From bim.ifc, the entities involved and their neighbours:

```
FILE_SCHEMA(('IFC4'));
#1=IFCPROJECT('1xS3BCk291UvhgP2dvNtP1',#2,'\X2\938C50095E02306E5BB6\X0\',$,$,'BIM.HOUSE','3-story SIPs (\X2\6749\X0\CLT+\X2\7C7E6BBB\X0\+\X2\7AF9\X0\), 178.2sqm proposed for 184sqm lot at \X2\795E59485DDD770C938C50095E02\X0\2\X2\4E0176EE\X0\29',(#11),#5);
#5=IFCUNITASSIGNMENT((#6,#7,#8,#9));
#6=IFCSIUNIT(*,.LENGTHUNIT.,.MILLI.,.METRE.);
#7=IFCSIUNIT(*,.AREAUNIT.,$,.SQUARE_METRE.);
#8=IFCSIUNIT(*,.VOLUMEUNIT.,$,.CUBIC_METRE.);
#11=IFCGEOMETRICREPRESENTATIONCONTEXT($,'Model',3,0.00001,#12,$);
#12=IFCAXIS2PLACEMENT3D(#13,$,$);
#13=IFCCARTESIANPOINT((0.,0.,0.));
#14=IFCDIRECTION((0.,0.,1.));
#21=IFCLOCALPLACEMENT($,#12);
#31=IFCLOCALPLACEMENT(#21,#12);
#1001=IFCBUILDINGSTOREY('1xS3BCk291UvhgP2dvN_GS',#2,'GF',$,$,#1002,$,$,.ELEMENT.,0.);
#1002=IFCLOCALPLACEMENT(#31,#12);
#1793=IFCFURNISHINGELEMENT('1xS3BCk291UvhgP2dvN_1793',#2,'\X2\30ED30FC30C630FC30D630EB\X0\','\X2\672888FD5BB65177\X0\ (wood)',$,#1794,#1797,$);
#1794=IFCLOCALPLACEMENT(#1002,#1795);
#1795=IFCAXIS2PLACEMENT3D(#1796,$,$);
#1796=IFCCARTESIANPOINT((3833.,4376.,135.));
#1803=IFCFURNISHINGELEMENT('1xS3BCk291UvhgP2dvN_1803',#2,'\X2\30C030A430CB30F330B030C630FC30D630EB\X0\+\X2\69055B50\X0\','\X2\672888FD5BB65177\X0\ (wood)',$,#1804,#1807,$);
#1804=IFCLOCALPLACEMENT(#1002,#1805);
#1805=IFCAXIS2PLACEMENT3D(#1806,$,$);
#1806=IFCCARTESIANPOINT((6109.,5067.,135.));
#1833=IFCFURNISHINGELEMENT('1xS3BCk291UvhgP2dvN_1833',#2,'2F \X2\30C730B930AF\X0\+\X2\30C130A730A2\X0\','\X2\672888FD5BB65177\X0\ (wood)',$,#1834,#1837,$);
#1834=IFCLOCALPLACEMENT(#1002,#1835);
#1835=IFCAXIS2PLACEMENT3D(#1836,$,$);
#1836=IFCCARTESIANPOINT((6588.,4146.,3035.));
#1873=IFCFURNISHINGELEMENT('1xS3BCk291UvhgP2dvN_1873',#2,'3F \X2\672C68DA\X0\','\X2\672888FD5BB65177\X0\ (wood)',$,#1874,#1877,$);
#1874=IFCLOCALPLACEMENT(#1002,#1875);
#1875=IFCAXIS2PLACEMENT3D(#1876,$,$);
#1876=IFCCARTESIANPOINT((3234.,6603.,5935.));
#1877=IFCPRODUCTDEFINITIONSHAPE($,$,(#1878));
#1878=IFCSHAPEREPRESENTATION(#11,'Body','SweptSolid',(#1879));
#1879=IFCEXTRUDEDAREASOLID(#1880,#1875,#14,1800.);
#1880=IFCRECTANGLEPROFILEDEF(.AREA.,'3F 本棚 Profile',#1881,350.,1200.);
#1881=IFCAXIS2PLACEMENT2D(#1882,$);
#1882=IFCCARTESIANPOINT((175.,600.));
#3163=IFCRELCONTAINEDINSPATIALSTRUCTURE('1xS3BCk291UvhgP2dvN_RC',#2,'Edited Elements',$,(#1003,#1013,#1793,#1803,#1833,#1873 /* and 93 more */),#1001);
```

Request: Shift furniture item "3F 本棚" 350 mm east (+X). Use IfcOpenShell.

```python
import ifcopenshell
import ifcopenshell.api.geometry
import ifcopenshell.util.placement

model = ifcopenshell.open("bim.ifc")

item = model.by_guid("1xS3BCk291UvhgP2dvN_1873")
matrix = ifcopenshell.util.placement.get_local_placement(item.ObjectPlacement)
matrix[0, 3] += 350.0
ifcopenshell.api.geometry.edit_object_placement(model, product=item, matrix=matrix, is_si=False)

print(ifcopenshell.util.placement.get_local_placement(item.ObjectPlacement).round(3) + 0.0)

model.write("bim_v2.ifc")
```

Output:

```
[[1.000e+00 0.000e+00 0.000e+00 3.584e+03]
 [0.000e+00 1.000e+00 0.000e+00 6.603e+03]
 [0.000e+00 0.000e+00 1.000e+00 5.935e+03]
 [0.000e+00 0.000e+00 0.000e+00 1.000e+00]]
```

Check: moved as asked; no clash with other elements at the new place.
